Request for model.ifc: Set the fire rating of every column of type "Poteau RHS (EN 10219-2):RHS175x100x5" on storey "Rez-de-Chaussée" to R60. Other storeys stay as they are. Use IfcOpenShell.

First a look at what the model holds.

```python
import ifcopenshell
import ifcopenshell.util.element

model = ifcopenshell.open("model.ifc")
print(model.schema)
storey = next(s for s in model.by_type("IfcBuildingStorey") if s.Name == "Rez-de-Chaussée")
columns = [e for e in ifcopenshell.util.element.get_decomposition(storey) if e.is_a("IfcColumn")]
seen = {}
for e in columns:
    element_type = ifcopenshell.util.element.get_type(e)
    key = (element_type.Name if element_type != e and element_type else None, ifcopenshell.util.element.get_pset(e, "Pset_ColumnCommon", "FireRating"))
    seen[key] = seen.get(key, 0) + 1
for (name, value), count in sorted(seen.items(), key=str):
    print(count, "x", name, "|", value)
```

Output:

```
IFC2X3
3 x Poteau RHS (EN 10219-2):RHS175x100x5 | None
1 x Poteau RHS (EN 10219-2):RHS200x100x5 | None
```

```python
import ifcopenshell
import ifcopenshell.api.pset
import ifcopenshell.util.element

model = ifcopenshell.open("model.ifc")

storey = next(s for s in model.by_type("IfcBuildingStorey") if s.Name == "Rez-de-Chaussée")
columns = [e for e in ifcopenshell.util.element.get_decomposition(storey) if e.is_a("IfcColumn")]

count = 0
for e in columns:
    element_type = ifcopenshell.util.element.get_type(e)
    if element_type in (None, e) or element_type.Name != "Poteau RHS (EN 10219-2):RHS175x100x5":
        continue
    # add_pset returns the element's existing set when there is one.
    pset = ifcopenshell.api.pset.add_pset(model, product=e, name="Pset_ColumnCommon")
    ifcopenshell.api.pset.edit_pset(model, pset=pset, properties={"FireRating": "R60"})
    count += 1

print(count, "columns updated")

model.write("model_edited.ifc")
```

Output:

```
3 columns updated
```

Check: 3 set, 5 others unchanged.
